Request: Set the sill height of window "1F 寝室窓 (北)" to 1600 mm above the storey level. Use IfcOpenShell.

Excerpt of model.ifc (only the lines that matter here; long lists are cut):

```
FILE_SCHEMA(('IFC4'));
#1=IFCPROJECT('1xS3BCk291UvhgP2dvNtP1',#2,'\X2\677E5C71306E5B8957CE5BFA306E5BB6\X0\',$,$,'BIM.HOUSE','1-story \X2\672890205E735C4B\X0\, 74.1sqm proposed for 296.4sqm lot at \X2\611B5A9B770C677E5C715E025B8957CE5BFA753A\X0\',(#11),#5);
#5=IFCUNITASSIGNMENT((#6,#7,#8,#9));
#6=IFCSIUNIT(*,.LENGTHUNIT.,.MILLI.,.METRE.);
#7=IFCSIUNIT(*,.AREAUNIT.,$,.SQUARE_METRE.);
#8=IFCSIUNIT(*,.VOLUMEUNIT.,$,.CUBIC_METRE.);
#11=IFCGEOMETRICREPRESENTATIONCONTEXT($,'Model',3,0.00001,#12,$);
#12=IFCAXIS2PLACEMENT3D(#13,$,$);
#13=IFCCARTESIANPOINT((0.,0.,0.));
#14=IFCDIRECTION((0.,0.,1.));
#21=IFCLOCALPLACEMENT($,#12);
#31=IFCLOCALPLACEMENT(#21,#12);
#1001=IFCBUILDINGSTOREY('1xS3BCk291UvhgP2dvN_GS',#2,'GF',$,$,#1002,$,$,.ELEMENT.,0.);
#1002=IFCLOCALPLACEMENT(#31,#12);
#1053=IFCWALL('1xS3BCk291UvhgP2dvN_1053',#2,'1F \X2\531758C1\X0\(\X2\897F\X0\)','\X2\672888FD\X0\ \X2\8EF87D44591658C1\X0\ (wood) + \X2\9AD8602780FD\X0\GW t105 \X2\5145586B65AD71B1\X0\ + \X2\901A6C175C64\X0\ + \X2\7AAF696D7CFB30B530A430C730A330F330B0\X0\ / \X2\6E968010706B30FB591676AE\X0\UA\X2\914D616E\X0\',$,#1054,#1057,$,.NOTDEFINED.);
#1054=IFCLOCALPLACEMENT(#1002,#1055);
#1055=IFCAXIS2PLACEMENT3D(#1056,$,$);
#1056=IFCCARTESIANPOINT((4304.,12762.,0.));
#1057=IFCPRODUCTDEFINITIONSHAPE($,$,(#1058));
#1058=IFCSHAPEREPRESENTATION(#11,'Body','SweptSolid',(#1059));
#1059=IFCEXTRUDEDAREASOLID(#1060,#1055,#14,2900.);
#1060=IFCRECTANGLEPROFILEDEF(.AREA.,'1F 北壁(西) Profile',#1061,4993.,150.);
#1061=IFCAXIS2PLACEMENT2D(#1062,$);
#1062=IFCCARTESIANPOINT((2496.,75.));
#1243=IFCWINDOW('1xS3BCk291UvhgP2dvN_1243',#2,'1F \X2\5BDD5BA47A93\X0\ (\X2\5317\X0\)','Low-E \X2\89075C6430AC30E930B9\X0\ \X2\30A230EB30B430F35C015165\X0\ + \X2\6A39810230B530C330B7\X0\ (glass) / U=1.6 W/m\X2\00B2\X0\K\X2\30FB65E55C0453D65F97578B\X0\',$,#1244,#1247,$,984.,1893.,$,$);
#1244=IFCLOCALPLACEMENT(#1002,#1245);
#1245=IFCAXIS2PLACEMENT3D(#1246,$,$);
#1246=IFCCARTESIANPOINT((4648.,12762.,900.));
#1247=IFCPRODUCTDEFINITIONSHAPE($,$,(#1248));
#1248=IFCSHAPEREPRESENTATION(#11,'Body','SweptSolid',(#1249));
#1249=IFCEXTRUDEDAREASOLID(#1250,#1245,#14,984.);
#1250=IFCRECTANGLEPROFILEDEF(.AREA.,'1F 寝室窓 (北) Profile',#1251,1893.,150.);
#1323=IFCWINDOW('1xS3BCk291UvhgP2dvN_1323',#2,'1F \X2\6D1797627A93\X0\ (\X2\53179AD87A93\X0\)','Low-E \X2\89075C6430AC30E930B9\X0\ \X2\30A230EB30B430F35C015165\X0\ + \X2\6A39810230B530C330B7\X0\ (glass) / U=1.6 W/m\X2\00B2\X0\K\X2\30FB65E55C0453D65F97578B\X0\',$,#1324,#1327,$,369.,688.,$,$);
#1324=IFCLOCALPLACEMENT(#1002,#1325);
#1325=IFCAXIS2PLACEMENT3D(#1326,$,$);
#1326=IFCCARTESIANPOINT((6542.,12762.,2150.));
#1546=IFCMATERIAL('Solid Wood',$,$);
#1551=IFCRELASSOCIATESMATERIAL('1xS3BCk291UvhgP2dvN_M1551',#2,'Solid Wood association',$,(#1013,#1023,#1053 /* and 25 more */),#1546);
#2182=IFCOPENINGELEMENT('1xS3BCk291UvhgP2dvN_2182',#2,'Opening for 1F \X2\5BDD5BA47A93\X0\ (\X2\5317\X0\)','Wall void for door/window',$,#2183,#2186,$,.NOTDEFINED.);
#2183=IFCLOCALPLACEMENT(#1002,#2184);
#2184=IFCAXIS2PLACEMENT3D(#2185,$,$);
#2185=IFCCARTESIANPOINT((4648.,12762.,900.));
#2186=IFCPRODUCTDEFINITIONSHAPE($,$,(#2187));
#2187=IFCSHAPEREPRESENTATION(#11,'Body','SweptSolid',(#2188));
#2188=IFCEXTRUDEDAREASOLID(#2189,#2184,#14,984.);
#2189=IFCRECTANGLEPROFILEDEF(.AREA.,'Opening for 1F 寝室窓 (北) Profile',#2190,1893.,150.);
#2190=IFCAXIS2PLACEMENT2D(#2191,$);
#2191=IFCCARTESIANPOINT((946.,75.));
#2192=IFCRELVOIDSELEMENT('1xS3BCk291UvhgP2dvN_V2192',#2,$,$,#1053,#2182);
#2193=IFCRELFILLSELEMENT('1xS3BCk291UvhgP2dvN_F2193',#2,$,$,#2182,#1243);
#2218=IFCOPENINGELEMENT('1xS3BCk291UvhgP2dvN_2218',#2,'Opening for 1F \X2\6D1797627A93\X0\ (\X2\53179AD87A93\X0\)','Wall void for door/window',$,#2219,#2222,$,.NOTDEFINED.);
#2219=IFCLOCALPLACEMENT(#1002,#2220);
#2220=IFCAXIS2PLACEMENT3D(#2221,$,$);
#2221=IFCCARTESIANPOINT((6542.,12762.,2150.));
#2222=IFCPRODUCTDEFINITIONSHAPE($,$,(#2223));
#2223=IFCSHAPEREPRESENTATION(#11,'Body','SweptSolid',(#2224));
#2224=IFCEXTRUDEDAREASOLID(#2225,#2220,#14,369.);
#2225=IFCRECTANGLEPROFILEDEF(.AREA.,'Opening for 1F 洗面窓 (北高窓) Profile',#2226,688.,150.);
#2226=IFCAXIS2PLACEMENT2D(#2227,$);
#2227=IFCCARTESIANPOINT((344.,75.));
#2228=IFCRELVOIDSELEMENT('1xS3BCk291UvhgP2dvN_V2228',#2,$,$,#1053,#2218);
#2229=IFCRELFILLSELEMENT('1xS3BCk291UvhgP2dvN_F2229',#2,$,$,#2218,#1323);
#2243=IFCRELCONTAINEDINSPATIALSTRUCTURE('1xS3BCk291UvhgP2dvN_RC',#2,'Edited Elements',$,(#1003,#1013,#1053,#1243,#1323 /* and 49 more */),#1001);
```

```python
import numpy as np
import ifcopenshell
import ifcopenshell.api.geometry
import ifcopenshell.geom
import ifcopenshell.util.element
import ifcopenshell.util.placement
import ifcopenshell.util.shape
import ifcopenshell.util.unit

model = ifcopenshell.open("model.ifc")
unit_scale = ifcopenshell.util.unit.calculate_unit_scale(model)

window = model.by_guid("1xS3BCk291UvhgP2dvN_1243")
opening = window.FillsVoids[0].RelatingOpeningElement
storey = ifcopenshell.util.element.get_container(window, ifc_class="IfcBuildingStorey")
level = ifcopenshell.util.placement.get_local_placement(storey.ObjectPlacement)[2, 3]

# The opening's origin need not be at the sill, so measure its lowest point.
shape = ifcopenshell.geom.create_shape(ifcopenshell.geom.settings(), opening)
bottom = ifcopenshell.util.shape.get_shape_bottom_elevation(shape, shape.geometry) / unit_scale
dz = level + 1.6 / unit_scale - bottom

shift = np.array([0.0, 0.0, dz])
# The window is not placed relative to its opening, so move both.
for product in (opening, window):
    matrix = ifcopenshell.util.placement.get_local_placement(product.ObjectPlacement)
    matrix[:3, 3] += shift
    ifcopenshell.api.geometry.edit_object_placement(model, product=product, matrix=matrix, is_si=False)

print(f"moved by {dz * unit_scale:+.3f} m")

model.write("model_v2.ifc")
```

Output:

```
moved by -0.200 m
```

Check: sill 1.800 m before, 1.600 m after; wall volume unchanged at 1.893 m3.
